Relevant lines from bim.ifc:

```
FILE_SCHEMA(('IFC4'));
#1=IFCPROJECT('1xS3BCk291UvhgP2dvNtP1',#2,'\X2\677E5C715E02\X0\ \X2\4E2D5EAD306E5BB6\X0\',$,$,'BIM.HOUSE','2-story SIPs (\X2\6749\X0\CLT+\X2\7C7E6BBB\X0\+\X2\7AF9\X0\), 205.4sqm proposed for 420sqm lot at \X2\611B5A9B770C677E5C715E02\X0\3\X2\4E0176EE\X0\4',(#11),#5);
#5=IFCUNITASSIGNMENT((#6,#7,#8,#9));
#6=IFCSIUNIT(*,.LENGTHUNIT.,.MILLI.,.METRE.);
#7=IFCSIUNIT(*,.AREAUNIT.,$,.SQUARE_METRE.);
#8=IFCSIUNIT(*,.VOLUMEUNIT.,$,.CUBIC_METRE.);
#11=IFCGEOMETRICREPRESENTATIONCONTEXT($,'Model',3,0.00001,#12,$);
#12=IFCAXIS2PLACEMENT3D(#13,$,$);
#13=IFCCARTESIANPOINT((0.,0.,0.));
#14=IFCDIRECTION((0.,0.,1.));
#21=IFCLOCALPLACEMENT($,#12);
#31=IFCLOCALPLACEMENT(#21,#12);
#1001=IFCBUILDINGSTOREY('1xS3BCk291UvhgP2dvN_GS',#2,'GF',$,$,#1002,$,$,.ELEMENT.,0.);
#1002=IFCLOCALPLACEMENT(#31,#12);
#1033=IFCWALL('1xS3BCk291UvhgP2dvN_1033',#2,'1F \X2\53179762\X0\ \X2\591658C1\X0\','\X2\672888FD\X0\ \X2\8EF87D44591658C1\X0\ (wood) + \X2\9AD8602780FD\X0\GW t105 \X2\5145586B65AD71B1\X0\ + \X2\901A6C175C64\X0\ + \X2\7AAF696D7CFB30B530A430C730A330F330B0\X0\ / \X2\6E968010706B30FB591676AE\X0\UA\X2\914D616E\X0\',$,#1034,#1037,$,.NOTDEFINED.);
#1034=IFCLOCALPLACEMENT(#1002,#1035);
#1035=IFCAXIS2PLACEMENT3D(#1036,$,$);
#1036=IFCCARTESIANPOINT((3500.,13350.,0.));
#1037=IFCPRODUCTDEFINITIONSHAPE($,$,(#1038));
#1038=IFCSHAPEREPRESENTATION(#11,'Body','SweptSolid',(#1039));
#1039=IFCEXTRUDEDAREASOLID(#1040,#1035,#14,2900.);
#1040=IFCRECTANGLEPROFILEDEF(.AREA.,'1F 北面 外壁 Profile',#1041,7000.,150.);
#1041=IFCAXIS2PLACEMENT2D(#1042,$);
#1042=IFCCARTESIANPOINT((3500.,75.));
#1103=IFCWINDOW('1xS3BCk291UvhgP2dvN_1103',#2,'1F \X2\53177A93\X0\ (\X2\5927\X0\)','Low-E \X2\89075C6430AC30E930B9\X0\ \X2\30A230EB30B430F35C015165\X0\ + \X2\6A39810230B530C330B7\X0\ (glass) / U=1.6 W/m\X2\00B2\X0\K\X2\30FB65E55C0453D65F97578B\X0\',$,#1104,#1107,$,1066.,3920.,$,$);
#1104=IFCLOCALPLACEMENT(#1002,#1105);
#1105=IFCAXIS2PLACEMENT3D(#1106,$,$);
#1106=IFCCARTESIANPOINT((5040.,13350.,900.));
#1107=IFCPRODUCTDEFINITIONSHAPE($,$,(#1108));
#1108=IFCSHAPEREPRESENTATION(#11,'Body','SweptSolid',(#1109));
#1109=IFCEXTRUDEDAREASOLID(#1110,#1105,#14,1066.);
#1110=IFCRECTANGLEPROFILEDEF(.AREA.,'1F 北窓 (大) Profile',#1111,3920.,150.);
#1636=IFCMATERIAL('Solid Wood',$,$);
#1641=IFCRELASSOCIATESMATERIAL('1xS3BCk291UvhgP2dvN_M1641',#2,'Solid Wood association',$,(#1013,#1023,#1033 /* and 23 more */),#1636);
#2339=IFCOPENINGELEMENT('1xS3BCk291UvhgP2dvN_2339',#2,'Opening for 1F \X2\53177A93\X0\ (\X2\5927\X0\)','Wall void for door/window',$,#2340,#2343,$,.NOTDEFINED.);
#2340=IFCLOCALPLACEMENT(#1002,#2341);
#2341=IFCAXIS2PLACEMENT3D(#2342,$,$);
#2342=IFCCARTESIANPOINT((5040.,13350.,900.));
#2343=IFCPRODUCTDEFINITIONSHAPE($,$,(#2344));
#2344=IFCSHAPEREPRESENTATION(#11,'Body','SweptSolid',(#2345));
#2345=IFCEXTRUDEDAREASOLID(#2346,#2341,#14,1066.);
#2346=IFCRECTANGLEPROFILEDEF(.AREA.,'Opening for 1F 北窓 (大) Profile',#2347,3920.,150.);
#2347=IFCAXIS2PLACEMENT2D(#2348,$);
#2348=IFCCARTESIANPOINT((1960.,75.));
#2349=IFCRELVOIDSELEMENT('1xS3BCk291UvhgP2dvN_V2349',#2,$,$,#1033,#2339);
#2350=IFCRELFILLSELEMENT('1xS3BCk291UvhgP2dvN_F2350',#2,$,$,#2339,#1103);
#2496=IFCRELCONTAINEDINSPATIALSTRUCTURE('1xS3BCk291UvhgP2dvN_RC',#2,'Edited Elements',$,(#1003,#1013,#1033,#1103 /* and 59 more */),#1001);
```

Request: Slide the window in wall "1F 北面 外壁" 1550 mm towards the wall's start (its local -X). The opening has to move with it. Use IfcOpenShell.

```python
import ifcopenshell
import ifcopenshell.api.geometry
import ifcopenshell.util.placement
import ifcopenshell.util.unit

model = ifcopenshell.open("bim.ifc")
unit_scale = ifcopenshell.util.unit.calculate_unit_scale(model)

window = model.by_guid("1xS3BCk291UvhgP2dvN_1103")
opening = window.FillsVoids[0].RelatingOpeningElement
wall = opening.VoidsElements[0].RelatingBuildingElement

wall_matrix = ifcopenshell.util.placement.get_local_placement(wall.ObjectPlacement)
shift = wall_matrix[:3, 0] * -1.55 / unit_scale
before = ifcopenshell.util.placement.get_local_placement(window.ObjectPlacement)[:3, 3].copy()

# The window is not placed relative to its opening, so move both.
for product in (opening, window):
    matrix = ifcopenshell.util.placement.get_local_placement(product.ObjectPlacement)
    matrix[:3, 3] += shift
    ifcopenshell.api.geometry.edit_object_placement(model, product=product, matrix=matrix, is_si=False)

after = ifcopenshell.util.placement.get_local_placement(window.ObjectPlacement)[:3, 3]
print("window moved by", (after - before).round(3) + 0.0)

model.write("bim_edited.ifc")
```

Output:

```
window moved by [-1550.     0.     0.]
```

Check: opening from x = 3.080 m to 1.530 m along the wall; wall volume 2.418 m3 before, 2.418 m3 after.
